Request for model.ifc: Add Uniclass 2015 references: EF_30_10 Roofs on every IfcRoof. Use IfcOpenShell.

First a look at what the model holds.

```python
import ifcopenshell

model = ifcopenshell.open("model.ifc")
print(model.schema)
print("classifications:", [c.Name for c in model.by_type("IfcClassification")])
for ifc_class in ("IfcDoor", "IfcRoof", "IfcStair", "IfcWall", "IfcWindow"):
    print(ifc_class, len(model.by_type(ifc_class)))
```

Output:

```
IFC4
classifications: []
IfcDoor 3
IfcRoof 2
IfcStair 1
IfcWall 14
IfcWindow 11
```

```python
import ifcopenshell
import ifcopenshell.api.classification

model = ifcopenshell.open("model.ifc")

system = ifcopenshell.api.classification.add_classification(model, classification="Uniclass 2015")

codes = {
    "IfcRoof": ("EF_30_10", "Roofs"),
}
for ifc_class, (code, name) in codes.items():
    products = model.by_type(ifc_class)
    ifcopenshell.api.classification.add_reference(
        model, products=products, classification=system, identification=code, name=name
    )
    print(code, len(products))

model.write("model_rev.ifc")
```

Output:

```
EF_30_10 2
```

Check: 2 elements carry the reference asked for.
